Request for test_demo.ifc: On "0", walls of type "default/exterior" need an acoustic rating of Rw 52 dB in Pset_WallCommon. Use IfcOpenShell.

First a look at what the model holds.

```python
import ifcopenshell
import ifcopenshell.util.element

model = ifcopenshell.open("test_demo.ifc")
print(model.schema)
storey = next(s for s in model.by_type("IfcBuildingStorey") if s.Name == "0")
walls = [e for e in ifcopenshell.util.element.get_decomposition(storey) if e.is_a("IfcWall")]
seen = {}
for e in walls:
    element_type = ifcopenshell.util.element.get_type(e)
    key = (element_type.Name if element_type != e and element_type else None, ifcopenshell.util.element.get_pset(e, "Pset_WallCommon", "AcousticRating"))
    seen[key] = seen.get(key, 0) + 1
for (name, value), count in sorted(seen.items(), key=str):
    print(count, "x", name, "|", value)
```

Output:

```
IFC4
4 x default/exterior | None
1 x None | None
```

```python
import ifcopenshell
import ifcopenshell.api.pset
import ifcopenshell.util.element

model = ifcopenshell.open("test_demo.ifc")

storey = next(s for s in model.by_type("IfcBuildingStorey") if s.Name == "0")
walls = [e for e in ifcopenshell.util.element.get_decomposition(storey) if e.is_a("IfcWall")]

count = 0
for e in walls:
    element_type = ifcopenshell.util.element.get_type(e)
    if element_type in (None, e) or element_type.Name != "default/exterior":
        continue
    # add_pset returns the element's existing set when there is one.
    pset = ifcopenshell.api.pset.add_pset(model, product=e, name="Pset_WallCommon")
    ifcopenshell.api.pset.edit_pset(model, pset=pset, properties={"AcousticRating": "Rw 52 dB"})
    count += 1

print(count, "walls updated")

model.write("test_demo_v2.ifc")
```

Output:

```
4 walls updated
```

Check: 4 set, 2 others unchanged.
